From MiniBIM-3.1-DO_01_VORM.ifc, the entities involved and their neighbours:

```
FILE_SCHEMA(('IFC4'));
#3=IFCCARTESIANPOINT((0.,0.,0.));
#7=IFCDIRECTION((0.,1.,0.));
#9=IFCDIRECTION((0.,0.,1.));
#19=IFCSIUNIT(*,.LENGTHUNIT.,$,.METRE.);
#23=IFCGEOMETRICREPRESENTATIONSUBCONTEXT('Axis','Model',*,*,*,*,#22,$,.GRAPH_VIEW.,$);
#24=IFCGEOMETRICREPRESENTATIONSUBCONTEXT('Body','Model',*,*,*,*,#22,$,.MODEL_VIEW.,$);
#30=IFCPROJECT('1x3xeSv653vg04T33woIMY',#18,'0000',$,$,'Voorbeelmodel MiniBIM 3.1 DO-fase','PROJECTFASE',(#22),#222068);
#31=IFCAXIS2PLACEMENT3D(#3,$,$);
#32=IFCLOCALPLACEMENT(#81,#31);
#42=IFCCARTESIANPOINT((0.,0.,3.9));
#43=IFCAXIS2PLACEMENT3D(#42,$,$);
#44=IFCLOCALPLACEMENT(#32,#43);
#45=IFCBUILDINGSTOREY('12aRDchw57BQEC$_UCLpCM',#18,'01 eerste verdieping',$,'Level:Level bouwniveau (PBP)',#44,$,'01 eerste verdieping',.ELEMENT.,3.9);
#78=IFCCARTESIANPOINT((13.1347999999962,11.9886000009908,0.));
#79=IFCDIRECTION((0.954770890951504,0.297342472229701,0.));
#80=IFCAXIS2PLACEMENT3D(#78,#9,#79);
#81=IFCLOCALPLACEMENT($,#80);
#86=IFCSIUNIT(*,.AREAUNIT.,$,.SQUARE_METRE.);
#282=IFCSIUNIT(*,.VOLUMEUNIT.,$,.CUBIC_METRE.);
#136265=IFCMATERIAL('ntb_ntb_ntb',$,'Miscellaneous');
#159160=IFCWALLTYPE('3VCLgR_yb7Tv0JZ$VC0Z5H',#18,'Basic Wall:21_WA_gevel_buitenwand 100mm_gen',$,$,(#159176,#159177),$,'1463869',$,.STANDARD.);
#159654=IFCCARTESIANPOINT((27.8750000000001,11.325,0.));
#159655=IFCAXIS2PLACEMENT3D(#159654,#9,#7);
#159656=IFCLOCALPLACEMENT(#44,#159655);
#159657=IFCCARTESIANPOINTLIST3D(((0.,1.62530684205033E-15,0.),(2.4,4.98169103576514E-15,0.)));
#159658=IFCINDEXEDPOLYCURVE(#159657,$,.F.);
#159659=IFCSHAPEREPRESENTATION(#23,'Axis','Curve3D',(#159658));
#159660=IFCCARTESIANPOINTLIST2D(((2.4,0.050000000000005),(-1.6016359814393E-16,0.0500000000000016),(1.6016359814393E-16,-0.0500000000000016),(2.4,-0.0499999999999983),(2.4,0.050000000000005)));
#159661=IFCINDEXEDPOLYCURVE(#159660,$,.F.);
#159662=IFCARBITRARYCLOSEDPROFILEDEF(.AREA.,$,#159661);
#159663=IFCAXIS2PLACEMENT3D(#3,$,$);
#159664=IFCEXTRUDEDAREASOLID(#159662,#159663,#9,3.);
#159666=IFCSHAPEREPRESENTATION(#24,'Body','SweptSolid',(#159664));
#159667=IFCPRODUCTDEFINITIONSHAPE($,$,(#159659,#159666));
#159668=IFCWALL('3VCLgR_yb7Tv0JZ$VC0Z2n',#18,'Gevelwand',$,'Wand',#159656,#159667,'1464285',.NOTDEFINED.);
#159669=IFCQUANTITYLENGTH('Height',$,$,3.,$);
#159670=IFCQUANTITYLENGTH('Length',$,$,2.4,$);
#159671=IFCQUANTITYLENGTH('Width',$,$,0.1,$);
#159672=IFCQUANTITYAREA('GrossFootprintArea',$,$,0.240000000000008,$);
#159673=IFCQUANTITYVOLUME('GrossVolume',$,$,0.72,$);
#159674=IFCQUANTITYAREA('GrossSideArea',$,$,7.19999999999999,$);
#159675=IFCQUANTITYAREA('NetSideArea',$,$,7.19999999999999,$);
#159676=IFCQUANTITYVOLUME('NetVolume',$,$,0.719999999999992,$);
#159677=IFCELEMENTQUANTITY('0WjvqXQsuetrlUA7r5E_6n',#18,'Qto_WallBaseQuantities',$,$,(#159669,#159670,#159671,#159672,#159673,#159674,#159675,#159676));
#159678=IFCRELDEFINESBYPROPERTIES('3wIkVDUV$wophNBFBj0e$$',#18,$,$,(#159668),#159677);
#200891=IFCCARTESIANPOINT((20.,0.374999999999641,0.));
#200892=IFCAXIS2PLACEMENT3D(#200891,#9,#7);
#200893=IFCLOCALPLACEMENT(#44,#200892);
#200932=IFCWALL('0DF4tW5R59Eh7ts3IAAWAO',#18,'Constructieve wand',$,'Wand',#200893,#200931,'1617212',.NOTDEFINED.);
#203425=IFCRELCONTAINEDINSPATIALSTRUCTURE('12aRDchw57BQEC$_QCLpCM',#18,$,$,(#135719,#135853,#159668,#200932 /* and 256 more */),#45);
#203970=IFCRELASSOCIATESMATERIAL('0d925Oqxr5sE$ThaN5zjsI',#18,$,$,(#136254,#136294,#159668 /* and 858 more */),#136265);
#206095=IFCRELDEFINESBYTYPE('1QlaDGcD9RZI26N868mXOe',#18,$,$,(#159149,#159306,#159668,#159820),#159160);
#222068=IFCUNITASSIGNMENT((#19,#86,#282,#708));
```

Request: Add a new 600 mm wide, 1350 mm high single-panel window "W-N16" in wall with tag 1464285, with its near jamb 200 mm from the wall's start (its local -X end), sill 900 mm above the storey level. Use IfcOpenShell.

```python
import numpy as np
import ifcopenshell
import ifcopenshell.api.feature
import ifcopenshell.api.geometry
import ifcopenshell.api.pset
import ifcopenshell.api.root
import ifcopenshell.api.spatial
import ifcopenshell.geom
import ifcopenshell.util.element
import ifcopenshell.util.placement
import ifcopenshell.util.representation
import ifcopenshell.util.shape
import ifcopenshell.util.unit

model = ifcopenshell.open("MiniBIM-3.1-DO_01_VORM.ifc")
unit_scale = ifcopenshell.util.unit.calculate_unit_scale(model)
area_scale = ifcopenshell.util.unit.calculate_unit_scale(model, "AREAUNIT")
volume_scale = ifcopenshell.util.unit.calculate_unit_scale(model, "VOLUMEUNIT")
settings = ifcopenshell.geom.settings()


def volume(element):
    """Net volume in cubic metres, openings subtracted."""
    shape = ifcopenshell.geom.create_shape(settings, element)
    return ifcopenshell.util.shape.get_volume(shape.geometry)


wall = model.by_id(159668)
storey = ifcopenshell.util.element.get_container(wall, ifc_class="IfcBuildingStorey")
context = ifcopenshell.util.representation.get_context(model, "Model", "Body", "MODEL_VIEW")
before = volume(wall)

width, height, from_end, sill = 0.6, 1.35, 0.2, 0.9  # metres

# The wall runs along its own X axis, and the end named is its -X end.
wall_shape = ifcopenshell.geom.create_shape(settings, wall)
x, y, z = ifcopenshell.util.shape.get_vertices(wall_shape.geometry).T
start = x.min() + from_end
face, thickness = float(y.min()), float(y.max() - y.min())
wall_matrix = ifcopenshell.util.placement.get_local_placement(wall.ObjectPlacement)
level = ifcopenshell.util.placement.get_local_placement(storey.ObjectPlacement)[2, 3]


def in_wall(x, y):
    """Placement at x, y metres in the wall's axes, at sill height."""
    matrix = wall_matrix.copy()
    matrix[:, 3] = wall_matrix @ np.array([x / unit_scale, y / unit_scale, 0.0, 1.0])
    matrix[2, 3] = level + sill / unit_scale
    return matrix


# Opening: a box that overshoots both wall faces by 50 mm.
opening = ifcopenshell.api.root.create_entity(model, ifc_class="IfcOpeningElement", predefined_type="OPENING")
box = ifcopenshell.api.geometry.add_wall_representation(
    model, context=context, length=width, height=height, thickness=thickness + 0.1
)
ifcopenshell.api.geometry.assign_representation(model, product=opening, representation=box)
ifcopenshell.api.geometry.edit_object_placement(model, product=opening, matrix=in_wall(start, face - 0.05), is_si=False)
ifcopenshell.api.feature.add_feature(model, feature=opening, element=wall)

window = ifcopenshell.api.root.create_entity(model, ifc_class="IfcWindow", name="W-N16", predefined_type="WINDOW")
window.OverallWidth, window.OverallHeight = width / unit_scale, height / unit_scale
window.PartitioningType = "SINGLE_PANEL"
body = ifcopenshell.api.geometry.add_window_representation(
    model,
    context=context,
    overall_width=window.OverallWidth,
    overall_height=window.OverallHeight,
    partition_type="SINGLE_PANEL",
)
ifcopenshell.api.geometry.assign_representation(model, product=window, representation=body)
ifcopenshell.api.spatial.assign_container(model, products=[window], relating_structure=storey)
ifcopenshell.api.feature.add_filling(model, opening=opening, element=window)

# Centre the window in the wall's thickness.
ifcopenshell.api.geometry.edit_object_placement(model, product=window, matrix=in_wall(start, face), is_si=False)
window_shape = ifcopenshell.geom.create_shape(settings, window)
depth = ifcopenshell.util.shape.get_vertices(window_shape.geometry)[:, 1]
offset = face + thickness / 2 - (depth.min() + depth.max()) / 2
ifcopenshell.api.geometry.edit_object_placement(model, product=window, matrix=in_wall(start, offset), is_si=False)

after = volume(wall)

# Update the wall's stored quantities.
qto = model.by_id(ifcopenshell.util.element.get_pset(wall, "Qto_WallBaseQuantities", should_inherit=False)["id"])
ifcopenshell.api.pset.edit_qto(model, qto=qto, properties={
    "NetSideArea": after / thickness / area_scale,
    "NetVolume": after / volume_scale,
})

print(f"wall volume {before:.3f} -> {after:.3f} m3")

model.write("MiniBIM-3.1-DO_01_VORM_edited.ifc")
```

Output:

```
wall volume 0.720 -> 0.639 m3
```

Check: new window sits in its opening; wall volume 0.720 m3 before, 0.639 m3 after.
